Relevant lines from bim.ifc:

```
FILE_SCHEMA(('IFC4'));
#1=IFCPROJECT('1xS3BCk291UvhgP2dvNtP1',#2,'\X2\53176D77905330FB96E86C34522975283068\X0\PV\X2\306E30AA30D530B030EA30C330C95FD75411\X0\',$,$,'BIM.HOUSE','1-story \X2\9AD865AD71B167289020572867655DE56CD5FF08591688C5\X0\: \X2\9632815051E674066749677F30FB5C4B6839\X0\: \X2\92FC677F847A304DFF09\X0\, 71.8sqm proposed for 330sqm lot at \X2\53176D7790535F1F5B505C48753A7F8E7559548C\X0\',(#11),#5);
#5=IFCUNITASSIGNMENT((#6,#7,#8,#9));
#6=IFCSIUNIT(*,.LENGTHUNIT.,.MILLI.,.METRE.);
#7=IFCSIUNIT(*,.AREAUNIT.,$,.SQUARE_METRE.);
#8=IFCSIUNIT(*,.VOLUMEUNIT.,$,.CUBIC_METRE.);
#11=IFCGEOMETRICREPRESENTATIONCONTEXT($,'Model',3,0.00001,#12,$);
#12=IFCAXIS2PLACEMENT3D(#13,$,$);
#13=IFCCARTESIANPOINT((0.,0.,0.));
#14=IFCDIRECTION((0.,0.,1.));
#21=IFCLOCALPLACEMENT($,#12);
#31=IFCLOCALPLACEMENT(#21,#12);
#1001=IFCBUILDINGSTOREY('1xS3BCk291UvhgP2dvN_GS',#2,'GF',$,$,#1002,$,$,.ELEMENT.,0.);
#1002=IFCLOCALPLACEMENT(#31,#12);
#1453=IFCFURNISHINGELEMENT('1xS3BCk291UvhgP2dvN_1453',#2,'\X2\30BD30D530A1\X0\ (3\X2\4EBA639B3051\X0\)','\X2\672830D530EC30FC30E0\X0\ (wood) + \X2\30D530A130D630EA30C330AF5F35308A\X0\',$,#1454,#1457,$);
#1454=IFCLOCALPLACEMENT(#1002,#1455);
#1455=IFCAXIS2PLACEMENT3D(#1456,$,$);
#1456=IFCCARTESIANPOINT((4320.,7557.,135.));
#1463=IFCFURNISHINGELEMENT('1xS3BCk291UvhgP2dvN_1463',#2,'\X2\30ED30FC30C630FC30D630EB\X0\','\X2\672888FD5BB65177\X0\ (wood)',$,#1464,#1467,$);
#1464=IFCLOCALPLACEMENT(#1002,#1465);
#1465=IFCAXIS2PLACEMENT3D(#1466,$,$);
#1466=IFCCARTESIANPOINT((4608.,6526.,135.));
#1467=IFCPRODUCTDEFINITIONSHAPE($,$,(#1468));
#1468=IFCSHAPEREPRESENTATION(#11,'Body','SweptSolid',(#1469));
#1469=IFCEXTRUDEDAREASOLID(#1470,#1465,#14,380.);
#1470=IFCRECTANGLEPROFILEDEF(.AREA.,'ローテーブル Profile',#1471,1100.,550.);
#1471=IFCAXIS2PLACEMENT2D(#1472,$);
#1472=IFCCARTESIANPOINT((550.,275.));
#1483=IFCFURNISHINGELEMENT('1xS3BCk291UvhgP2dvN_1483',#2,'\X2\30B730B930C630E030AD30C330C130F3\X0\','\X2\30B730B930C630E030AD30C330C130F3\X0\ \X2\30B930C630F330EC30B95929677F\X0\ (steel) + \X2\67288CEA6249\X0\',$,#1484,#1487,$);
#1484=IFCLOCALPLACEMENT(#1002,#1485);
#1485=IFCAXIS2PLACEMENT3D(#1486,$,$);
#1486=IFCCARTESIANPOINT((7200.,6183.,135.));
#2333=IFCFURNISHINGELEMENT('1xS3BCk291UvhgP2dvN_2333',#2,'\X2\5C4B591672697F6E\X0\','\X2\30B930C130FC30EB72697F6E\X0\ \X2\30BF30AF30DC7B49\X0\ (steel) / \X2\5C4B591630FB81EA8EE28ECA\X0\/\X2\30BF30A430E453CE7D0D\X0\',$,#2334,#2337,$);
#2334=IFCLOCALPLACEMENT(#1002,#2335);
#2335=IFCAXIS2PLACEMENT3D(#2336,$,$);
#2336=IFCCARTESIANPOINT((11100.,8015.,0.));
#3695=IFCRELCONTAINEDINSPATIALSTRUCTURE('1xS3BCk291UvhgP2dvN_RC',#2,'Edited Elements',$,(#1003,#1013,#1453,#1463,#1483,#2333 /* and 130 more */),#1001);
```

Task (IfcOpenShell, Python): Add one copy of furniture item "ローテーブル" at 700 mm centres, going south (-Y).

```python
import numpy as np
import ifcopenshell
import ifcopenshell.api.geometry
import ifcopenshell.api.root
import ifcopenshell.util.element
import ifcopenshell.util.placement
import ifcopenshell.util.unit

model = ifcopenshell.open("bim.ifc")
unit_scale = ifcopenshell.util.unit.calculate_unit_scale(model)


def reuse_history(source, copy):
    """copy_class also copies each property set's owner history, people and application; keep the originals."""
    for rel in copy.IsDefinedBy:
        if rel.is_a("IfcRelDefinesByProperties") and (history := rel.RelatingPropertyDefinition.OwnerHistory):
            rel.RelatingPropertyDefinition.OwnerHistory = source.OwnerHistory
            ifcopenshell.util.element.remove_deep2(model, history)


source = model.by_guid("1xS3BCk291UvhgP2dvN_1463")
base = ifcopenshell.util.placement.get_local_placement(source.ObjectPlacement)
step = np.array([0.0, -1.0, 0.0]) * 0.7 / unit_scale

for i in range(1, 2):
    copy = ifcopenshell.api.root.copy_class(model, product=source)
    copy.Representation = ifcopenshell.util.element.copy_deep(
        model, source.Representation, exclude=["IfcGeometricRepresentationContext", "IfcRepresentationMap"]
    )
    reuse_history(source, copy)
    matrix = base.copy()
    matrix[:3, 3] += i * step
    print("added at", matrix[:3, 3].round(3) + 0.0)
    ifcopenshell.api.geometry.edit_object_placement(model, product=copy, matrix=matrix, is_si=False)

model.write("bim_rev.ifc")
```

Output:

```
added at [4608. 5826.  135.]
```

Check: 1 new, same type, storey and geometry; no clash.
